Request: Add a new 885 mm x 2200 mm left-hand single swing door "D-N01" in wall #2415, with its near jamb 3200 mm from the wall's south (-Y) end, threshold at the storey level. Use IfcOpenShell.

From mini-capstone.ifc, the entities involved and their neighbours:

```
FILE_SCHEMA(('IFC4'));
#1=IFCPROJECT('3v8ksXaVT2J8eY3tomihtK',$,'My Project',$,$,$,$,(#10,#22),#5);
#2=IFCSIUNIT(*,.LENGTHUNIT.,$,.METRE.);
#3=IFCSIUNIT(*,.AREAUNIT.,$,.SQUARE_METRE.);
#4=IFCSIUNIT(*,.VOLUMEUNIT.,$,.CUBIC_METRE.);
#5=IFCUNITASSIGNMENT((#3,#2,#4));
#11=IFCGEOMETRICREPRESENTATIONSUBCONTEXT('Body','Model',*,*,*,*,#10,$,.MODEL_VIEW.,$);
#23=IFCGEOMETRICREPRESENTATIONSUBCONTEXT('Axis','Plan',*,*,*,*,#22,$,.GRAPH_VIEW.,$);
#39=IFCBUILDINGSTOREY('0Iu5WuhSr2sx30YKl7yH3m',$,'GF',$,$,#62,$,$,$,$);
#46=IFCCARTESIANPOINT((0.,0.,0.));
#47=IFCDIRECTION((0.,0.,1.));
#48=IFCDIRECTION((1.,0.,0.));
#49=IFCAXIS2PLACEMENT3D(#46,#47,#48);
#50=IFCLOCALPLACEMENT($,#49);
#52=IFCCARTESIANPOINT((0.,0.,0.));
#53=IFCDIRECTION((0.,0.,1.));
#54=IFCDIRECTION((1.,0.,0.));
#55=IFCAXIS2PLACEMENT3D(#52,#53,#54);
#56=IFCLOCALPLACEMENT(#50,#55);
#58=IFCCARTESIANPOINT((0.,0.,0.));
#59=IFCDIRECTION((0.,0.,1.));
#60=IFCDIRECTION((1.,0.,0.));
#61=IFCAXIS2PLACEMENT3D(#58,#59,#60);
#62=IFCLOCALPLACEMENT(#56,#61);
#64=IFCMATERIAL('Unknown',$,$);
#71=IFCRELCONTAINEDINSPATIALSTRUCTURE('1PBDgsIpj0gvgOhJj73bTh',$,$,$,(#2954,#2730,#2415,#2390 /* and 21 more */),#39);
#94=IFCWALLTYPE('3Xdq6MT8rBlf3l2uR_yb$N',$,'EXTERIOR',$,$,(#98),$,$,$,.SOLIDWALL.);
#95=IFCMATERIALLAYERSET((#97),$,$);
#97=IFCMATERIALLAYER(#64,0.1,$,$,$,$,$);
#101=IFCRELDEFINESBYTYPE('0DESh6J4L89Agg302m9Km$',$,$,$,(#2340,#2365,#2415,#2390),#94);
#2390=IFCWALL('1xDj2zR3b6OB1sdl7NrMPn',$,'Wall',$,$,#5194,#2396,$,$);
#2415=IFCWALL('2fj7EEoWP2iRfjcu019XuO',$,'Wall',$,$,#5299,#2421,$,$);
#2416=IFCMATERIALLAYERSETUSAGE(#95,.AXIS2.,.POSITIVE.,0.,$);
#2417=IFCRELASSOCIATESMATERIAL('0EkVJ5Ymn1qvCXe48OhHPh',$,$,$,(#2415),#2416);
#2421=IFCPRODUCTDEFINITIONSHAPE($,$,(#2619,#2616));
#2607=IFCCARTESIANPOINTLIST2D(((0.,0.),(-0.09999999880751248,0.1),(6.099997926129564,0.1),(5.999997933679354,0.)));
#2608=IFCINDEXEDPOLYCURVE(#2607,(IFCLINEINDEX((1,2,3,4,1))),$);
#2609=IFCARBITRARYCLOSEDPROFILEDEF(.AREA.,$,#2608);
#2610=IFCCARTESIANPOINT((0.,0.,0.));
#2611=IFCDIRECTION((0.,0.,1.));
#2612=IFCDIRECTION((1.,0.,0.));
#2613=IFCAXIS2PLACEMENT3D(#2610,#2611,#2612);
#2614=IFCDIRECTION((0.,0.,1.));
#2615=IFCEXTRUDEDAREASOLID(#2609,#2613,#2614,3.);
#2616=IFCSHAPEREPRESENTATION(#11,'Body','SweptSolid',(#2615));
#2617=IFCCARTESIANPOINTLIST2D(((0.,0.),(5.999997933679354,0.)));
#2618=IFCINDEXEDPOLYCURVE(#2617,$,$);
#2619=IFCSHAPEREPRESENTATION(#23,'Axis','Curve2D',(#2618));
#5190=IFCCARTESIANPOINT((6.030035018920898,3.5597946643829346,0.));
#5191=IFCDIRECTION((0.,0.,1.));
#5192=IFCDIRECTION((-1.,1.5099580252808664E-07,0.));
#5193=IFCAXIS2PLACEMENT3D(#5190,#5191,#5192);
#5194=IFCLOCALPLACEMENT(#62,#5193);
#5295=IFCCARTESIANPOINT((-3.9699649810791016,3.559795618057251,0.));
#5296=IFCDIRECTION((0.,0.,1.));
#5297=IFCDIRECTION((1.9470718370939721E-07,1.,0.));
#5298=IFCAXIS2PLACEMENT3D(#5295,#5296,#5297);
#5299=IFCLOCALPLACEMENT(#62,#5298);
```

```python
import numpy as np
import ifcopenshell
import ifcopenshell.api.feature
import ifcopenshell.api.geometry
import ifcopenshell.api.root
import ifcopenshell.api.spatial
import ifcopenshell.geom
import ifcopenshell.util.element
import ifcopenshell.util.placement
import ifcopenshell.util.representation
import ifcopenshell.util.shape
import ifcopenshell.util.unit

model = ifcopenshell.open("mini-capstone.ifc")
unit_scale = ifcopenshell.util.unit.calculate_unit_scale(model)
settings = ifcopenshell.geom.settings()


def volume(element):
    """Net volume in cubic metres, openings subtracted."""
    shape = ifcopenshell.geom.create_shape(settings, element)
    return ifcopenshell.util.shape.get_volume(shape.geometry)


wall = model.by_id(2415)
storey = ifcopenshell.util.element.get_container(wall, ifc_class="IfcBuildingStorey")
context = ifcopenshell.util.representation.get_context(model, "Model", "Body", "MODEL_VIEW")
before = volume(wall)

width, height, from_end, sill = 0.885, 2.2, 3.2, 0.0  # metres

# The wall runs along its own X axis, and the end named is its -X end.
wall_shape = ifcopenshell.geom.create_shape(settings, wall)
x, y, z = ifcopenshell.util.shape.get_vertices(wall_shape.geometry).T
start = x.min() + from_end
face, thickness = float(y.min()), float(y.max() - y.min())
wall_matrix = ifcopenshell.util.placement.get_local_placement(wall.ObjectPlacement)
level = ifcopenshell.util.placement.get_local_placement(storey.ObjectPlacement)[2, 3]


def in_wall(x, y):
    """Placement at x, y metres in the wall's axes, at sill height."""
    matrix = wall_matrix.copy()
    matrix[:, 3] = wall_matrix @ np.array([x / unit_scale, y / unit_scale, 0.0, 1.0])
    matrix[2, 3] = level + sill / unit_scale
    return matrix


# Opening: a box that overshoots both wall faces by 50 mm.
opening = ifcopenshell.api.root.create_entity(model, ifc_class="IfcOpeningElement", predefined_type="OPENING")
box = ifcopenshell.api.geometry.add_wall_representation(
    model, context=context, length=width, height=height, thickness=thickness + 0.1
)
ifcopenshell.api.geometry.assign_representation(model, product=opening, representation=box)
ifcopenshell.api.geometry.edit_object_placement(model, product=opening, matrix=in_wall(start, face - 0.05), is_si=False)
ifcopenshell.api.feature.add_feature(model, feature=opening, element=wall)

door = ifcopenshell.api.root.create_entity(model, ifc_class="IfcDoor", name="D-N01", predefined_type="DOOR")
door.OverallWidth, door.OverallHeight = width / unit_scale, height / unit_scale
door.OperationType = "SINGLE_SWING_LEFT"
body = ifcopenshell.api.geometry.add_door_representation(
    model,
    context=context,
    overall_width=door.OverallWidth,
    overall_height=door.OverallHeight,
    operation_type="SINGLE_SWING_LEFT",
    lining_properties={"LiningDepth": thickness / unit_scale, "ThresholdDepth": thickness / unit_scale},
)
ifcopenshell.api.geometry.assign_representation(model, product=door, representation=body)
ifcopenshell.api.spatial.assign_container(model, products=[door], relating_structure=storey)
ifcopenshell.api.feature.add_filling(model, opening=opening, element=door)

# The lining spans the wall, so the door starts at the wall face.
ifcopenshell.api.geometry.edit_object_placement(model, product=door, matrix=in_wall(start, face), is_si=False)

after = volume(wall)

print(f"wall volume {before:.3f} -> {after:.3f} m3")

model.write("mini-capstone-out.ifc")
```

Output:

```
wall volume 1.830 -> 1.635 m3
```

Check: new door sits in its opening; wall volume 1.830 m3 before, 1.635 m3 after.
